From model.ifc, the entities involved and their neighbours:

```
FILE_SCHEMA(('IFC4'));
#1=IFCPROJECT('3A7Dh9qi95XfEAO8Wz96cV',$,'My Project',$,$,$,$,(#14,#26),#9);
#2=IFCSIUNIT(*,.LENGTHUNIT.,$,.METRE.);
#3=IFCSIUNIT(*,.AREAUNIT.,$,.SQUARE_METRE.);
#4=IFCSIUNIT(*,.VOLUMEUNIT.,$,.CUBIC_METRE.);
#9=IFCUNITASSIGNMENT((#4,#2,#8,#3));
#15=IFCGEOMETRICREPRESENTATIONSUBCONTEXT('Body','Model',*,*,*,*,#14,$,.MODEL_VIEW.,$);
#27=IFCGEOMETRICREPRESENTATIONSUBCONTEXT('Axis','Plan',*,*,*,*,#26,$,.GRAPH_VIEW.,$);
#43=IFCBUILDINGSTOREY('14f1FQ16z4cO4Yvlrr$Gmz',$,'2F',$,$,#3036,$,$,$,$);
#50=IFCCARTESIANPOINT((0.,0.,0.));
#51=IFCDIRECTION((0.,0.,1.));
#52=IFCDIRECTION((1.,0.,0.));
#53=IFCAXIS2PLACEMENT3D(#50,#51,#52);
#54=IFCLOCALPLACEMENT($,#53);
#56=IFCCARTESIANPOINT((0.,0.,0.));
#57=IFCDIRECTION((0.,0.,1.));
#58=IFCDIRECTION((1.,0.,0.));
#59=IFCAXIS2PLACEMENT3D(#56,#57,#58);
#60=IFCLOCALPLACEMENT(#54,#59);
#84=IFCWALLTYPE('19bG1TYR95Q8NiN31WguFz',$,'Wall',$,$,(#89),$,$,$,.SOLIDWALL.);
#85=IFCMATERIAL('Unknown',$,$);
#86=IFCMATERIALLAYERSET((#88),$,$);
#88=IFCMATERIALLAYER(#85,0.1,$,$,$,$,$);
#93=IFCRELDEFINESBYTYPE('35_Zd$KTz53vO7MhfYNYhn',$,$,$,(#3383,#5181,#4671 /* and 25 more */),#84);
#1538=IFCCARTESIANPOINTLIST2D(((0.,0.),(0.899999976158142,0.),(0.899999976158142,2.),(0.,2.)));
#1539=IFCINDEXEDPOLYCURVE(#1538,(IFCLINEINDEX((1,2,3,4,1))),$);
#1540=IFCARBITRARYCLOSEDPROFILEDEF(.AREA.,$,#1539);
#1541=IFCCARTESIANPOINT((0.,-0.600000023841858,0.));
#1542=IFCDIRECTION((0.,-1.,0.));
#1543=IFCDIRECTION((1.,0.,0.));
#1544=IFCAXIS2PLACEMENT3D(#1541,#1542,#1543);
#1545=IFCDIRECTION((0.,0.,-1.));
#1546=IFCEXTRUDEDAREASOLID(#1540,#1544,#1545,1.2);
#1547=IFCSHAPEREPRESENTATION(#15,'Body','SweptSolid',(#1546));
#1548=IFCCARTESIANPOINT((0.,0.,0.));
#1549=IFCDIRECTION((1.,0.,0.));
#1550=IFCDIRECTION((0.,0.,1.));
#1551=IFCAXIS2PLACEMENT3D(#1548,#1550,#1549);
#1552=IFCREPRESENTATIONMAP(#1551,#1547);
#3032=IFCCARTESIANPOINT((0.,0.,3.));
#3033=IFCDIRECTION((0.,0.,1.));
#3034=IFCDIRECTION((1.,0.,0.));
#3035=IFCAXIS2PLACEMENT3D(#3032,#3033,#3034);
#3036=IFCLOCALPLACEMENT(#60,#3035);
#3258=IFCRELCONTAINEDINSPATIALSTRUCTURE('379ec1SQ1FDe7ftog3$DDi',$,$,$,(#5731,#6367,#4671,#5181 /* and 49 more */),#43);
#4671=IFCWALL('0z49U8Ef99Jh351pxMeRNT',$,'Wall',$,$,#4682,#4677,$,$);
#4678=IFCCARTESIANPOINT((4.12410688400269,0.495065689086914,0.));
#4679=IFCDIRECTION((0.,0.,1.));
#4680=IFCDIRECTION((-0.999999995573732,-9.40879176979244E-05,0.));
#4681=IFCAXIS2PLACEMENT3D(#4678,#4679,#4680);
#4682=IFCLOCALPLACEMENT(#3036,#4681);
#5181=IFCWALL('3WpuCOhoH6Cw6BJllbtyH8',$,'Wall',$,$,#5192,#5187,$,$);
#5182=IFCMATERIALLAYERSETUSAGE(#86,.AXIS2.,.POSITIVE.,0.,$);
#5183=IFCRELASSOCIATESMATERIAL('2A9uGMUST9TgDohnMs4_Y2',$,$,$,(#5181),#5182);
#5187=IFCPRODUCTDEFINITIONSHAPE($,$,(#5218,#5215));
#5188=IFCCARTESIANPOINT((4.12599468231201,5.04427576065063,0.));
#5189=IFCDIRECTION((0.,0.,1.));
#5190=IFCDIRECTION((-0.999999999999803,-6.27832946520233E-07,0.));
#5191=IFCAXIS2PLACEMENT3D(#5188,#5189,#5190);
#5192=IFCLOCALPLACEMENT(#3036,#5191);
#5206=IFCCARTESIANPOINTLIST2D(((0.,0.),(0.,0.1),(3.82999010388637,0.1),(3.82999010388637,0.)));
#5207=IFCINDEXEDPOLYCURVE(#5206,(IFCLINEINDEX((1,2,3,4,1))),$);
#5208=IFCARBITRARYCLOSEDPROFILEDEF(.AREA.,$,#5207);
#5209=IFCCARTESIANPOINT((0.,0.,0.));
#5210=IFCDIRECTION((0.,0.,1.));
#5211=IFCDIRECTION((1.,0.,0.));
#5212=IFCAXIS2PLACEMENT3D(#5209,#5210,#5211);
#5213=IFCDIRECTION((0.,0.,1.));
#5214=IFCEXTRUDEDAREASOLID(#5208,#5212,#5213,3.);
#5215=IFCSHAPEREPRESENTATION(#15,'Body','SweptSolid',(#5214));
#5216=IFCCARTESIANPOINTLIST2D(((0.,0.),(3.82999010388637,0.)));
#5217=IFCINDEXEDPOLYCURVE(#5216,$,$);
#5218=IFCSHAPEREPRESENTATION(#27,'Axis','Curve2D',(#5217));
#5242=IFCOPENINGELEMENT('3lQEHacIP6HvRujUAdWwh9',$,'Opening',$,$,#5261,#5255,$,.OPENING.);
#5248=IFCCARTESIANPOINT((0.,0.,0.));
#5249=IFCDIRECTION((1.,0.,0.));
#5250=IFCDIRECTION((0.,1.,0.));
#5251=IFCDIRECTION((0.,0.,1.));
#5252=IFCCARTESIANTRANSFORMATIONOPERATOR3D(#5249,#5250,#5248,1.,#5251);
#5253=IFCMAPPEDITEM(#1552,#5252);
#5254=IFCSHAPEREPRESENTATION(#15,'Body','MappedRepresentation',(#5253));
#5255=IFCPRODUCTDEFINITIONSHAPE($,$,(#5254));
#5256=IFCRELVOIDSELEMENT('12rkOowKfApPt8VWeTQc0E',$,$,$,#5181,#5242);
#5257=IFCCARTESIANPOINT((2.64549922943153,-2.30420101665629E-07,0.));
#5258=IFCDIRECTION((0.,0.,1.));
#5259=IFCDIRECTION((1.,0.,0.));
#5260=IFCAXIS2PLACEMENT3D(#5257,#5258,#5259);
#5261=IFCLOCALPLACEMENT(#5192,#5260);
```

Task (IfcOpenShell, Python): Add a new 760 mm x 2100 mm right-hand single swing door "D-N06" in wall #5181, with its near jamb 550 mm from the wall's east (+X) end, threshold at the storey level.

```python
import numpy as np
import ifcopenshell
import ifcopenshell.api.feature
import ifcopenshell.api.geometry
import ifcopenshell.api.root
import ifcopenshell.api.spatial
import ifcopenshell.geom
import ifcopenshell.util.element
import ifcopenshell.util.placement
import ifcopenshell.util.representation
import ifcopenshell.util.shape
import ifcopenshell.util.unit

model = ifcopenshell.open("model.ifc")
unit_scale = ifcopenshell.util.unit.calculate_unit_scale(model)
settings = ifcopenshell.geom.settings()


def volume(element):
    """Net volume in cubic metres, openings subtracted."""
    shape = ifcopenshell.geom.create_shape(settings, element)
    return ifcopenshell.util.shape.get_volume(shape.geometry)


wall = model.by_guid("3WpuCOhoH6Cw6BJllbtyH8")
storey = ifcopenshell.util.element.get_container(wall, ifc_class="IfcBuildingStorey")
context = ifcopenshell.util.representation.get_context(model, "Model", "Body", "MODEL_VIEW")
before = volume(wall)

width, height, from_end, sill = 0.76, 2.1, 0.55, 0.0  # metres

# The wall runs along its own X axis, and the end named is its -X end.
wall_shape = ifcopenshell.geom.create_shape(settings, wall)
x, y, z = ifcopenshell.util.shape.get_vertices(wall_shape.geometry).T
start = x.min() + from_end
face, thickness = float(y.min()), float(y.max() - y.min())
wall_matrix = ifcopenshell.util.placement.get_local_placement(wall.ObjectPlacement)
level = ifcopenshell.util.placement.get_local_placement(storey.ObjectPlacement)[2, 3]


def in_wall(x, y):
    """Placement at x, y metres in the wall's axes, at sill height."""
    matrix = wall_matrix.copy()
    matrix[:, 3] = wall_matrix @ np.array([x / unit_scale, y / unit_scale, 0.0, 1.0])
    matrix[2, 3] = level + sill / unit_scale
    return matrix


# Opening: a box that overshoots both wall faces by 50 mm.
opening = ifcopenshell.api.root.create_entity(model, ifc_class="IfcOpeningElement", predefined_type="OPENING")
box = ifcopenshell.api.geometry.add_wall_representation(
    model, context=context, length=width, height=height, thickness=thickness + 0.1
)
ifcopenshell.api.geometry.assign_representation(model, product=opening, representation=box)
ifcopenshell.api.geometry.edit_object_placement(model, product=opening, matrix=in_wall(start, face - 0.05), is_si=False)
ifcopenshell.api.feature.add_feature(model, feature=opening, element=wall)

door = ifcopenshell.api.root.create_entity(model, ifc_class="IfcDoor", name="D-N06", predefined_type="DOOR")
door.OverallWidth, door.OverallHeight = width / unit_scale, height / unit_scale
door.OperationType = "SINGLE_SWING_RIGHT"
body = ifcopenshell.api.geometry.add_door_representation(
    model,
    context=context,
    overall_width=door.OverallWidth,
    overall_height=door.OverallHeight,
    operation_type="SINGLE_SWING_RIGHT",
    lining_properties={"LiningDepth": thickness / unit_scale, "ThresholdDepth": thickness / unit_scale},
)
ifcopenshell.api.geometry.assign_representation(model, product=door, representation=body)
ifcopenshell.api.spatial.assign_container(model, products=[door], relating_structure=storey)
ifcopenshell.api.feature.add_filling(model, opening=opening, element=door)

# The lining spans the wall, so the door starts at the wall face.
ifcopenshell.api.geometry.edit_object_placement(model, product=door, matrix=in_wall(start, face), is_si=False)

after = volume(wall)

print(f"wall volume {before:.3f} -> {after:.3f} m3")

model.write("model-out.ifc")
```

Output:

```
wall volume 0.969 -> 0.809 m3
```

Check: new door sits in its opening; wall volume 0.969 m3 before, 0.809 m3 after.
